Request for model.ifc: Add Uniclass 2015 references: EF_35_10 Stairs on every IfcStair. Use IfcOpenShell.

First a look at what the model holds.

```python
import ifcopenshell

model = ifcopenshell.open("model.ifc")
print(model.schema)
print("classifications:", [c.Name for c in model.by_type("IfcClassification")])
for ifc_class in ("IfcDoor", "IfcRoof", "IfcStair", "IfcWall", "IfcWindow"):
    print(ifc_class, len(model.by_type(ifc_class)))
```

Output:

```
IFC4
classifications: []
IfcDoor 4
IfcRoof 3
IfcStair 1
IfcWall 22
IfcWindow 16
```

```python
import ifcopenshell
import ifcopenshell.api.classification

model = ifcopenshell.open("model.ifc")

system = ifcopenshell.api.classification.add_classification(model, classification="Uniclass 2015")

codes = {
    "IfcStair": ("EF_35_10", "Stairs"),
}
for ifc_class, (code, name) in codes.items():
    products = model.by_type(ifc_class)
    ifcopenshell.api.classification.add_reference(
        model, products=products, classification=system, identification=code, name=name
    )
    print(code, len(products))

model.write("model_updated.ifc")
```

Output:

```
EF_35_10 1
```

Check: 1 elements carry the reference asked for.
